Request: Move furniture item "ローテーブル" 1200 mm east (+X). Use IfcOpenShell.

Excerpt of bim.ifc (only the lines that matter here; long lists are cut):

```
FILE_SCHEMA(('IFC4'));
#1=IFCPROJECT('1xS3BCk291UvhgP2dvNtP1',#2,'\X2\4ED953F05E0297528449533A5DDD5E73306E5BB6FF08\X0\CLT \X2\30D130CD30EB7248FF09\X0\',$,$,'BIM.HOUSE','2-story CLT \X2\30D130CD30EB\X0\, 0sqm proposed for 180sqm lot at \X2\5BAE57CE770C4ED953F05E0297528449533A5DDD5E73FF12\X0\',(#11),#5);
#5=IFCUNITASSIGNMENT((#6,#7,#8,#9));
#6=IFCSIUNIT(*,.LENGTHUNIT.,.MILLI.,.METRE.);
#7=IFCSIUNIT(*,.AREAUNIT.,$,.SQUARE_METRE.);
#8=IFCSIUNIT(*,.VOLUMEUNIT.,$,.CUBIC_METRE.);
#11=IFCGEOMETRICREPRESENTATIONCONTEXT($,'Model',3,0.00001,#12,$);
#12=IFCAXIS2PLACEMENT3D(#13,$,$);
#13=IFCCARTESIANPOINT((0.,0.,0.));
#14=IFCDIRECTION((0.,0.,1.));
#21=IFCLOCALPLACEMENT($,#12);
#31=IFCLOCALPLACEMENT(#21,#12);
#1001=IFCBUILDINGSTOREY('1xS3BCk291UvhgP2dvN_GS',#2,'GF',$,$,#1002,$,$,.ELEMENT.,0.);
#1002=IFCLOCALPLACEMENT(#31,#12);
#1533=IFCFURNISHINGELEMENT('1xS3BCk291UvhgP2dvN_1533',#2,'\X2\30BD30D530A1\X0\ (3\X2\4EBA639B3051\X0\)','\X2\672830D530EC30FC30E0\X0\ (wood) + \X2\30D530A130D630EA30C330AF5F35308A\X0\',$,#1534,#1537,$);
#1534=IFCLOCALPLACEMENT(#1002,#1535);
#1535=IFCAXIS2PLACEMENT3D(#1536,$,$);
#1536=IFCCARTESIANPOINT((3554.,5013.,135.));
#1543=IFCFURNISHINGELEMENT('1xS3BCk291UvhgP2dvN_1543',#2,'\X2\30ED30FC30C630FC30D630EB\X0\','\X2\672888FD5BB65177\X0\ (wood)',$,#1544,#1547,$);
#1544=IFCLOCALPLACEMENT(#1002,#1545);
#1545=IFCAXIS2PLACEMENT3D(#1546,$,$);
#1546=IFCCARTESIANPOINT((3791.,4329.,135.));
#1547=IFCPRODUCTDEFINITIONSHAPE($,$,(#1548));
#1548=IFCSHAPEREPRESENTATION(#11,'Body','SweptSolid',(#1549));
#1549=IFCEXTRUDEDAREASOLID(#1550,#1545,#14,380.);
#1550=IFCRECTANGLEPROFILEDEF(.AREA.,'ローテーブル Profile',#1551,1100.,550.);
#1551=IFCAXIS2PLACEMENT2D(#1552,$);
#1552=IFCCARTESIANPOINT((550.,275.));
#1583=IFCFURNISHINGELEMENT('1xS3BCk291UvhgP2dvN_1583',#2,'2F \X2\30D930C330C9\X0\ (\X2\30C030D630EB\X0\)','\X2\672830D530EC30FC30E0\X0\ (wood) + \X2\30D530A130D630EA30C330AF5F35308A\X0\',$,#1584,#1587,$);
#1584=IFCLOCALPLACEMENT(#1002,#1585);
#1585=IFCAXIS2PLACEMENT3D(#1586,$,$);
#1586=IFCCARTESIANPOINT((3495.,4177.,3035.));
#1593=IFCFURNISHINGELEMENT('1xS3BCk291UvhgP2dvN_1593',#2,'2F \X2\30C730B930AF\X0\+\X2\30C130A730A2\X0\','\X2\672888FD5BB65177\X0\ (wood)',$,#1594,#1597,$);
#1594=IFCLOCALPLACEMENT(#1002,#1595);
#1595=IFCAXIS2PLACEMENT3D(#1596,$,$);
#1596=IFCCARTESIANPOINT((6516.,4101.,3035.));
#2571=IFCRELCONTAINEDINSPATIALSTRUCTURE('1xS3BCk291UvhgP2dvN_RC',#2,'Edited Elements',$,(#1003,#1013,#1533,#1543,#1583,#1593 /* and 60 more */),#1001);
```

```python
import ifcopenshell
import ifcopenshell.api.geometry
import ifcopenshell.util.placement

model = ifcopenshell.open("bim.ifc")

item = model.by_id(1543)
matrix = ifcopenshell.util.placement.get_local_placement(item.ObjectPlacement)
matrix[0, 3] += 1200.0
ifcopenshell.api.geometry.edit_object_placement(model, product=item, matrix=matrix, is_si=False)

print(ifcopenshell.util.placement.get_local_placement(item.ObjectPlacement).round(3) + 0.0)

model.write("bim_edited.ifc")
```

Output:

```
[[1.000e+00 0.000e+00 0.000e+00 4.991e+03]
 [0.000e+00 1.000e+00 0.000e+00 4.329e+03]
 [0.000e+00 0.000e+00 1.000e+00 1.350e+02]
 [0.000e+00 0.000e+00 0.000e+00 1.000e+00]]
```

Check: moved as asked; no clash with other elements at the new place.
